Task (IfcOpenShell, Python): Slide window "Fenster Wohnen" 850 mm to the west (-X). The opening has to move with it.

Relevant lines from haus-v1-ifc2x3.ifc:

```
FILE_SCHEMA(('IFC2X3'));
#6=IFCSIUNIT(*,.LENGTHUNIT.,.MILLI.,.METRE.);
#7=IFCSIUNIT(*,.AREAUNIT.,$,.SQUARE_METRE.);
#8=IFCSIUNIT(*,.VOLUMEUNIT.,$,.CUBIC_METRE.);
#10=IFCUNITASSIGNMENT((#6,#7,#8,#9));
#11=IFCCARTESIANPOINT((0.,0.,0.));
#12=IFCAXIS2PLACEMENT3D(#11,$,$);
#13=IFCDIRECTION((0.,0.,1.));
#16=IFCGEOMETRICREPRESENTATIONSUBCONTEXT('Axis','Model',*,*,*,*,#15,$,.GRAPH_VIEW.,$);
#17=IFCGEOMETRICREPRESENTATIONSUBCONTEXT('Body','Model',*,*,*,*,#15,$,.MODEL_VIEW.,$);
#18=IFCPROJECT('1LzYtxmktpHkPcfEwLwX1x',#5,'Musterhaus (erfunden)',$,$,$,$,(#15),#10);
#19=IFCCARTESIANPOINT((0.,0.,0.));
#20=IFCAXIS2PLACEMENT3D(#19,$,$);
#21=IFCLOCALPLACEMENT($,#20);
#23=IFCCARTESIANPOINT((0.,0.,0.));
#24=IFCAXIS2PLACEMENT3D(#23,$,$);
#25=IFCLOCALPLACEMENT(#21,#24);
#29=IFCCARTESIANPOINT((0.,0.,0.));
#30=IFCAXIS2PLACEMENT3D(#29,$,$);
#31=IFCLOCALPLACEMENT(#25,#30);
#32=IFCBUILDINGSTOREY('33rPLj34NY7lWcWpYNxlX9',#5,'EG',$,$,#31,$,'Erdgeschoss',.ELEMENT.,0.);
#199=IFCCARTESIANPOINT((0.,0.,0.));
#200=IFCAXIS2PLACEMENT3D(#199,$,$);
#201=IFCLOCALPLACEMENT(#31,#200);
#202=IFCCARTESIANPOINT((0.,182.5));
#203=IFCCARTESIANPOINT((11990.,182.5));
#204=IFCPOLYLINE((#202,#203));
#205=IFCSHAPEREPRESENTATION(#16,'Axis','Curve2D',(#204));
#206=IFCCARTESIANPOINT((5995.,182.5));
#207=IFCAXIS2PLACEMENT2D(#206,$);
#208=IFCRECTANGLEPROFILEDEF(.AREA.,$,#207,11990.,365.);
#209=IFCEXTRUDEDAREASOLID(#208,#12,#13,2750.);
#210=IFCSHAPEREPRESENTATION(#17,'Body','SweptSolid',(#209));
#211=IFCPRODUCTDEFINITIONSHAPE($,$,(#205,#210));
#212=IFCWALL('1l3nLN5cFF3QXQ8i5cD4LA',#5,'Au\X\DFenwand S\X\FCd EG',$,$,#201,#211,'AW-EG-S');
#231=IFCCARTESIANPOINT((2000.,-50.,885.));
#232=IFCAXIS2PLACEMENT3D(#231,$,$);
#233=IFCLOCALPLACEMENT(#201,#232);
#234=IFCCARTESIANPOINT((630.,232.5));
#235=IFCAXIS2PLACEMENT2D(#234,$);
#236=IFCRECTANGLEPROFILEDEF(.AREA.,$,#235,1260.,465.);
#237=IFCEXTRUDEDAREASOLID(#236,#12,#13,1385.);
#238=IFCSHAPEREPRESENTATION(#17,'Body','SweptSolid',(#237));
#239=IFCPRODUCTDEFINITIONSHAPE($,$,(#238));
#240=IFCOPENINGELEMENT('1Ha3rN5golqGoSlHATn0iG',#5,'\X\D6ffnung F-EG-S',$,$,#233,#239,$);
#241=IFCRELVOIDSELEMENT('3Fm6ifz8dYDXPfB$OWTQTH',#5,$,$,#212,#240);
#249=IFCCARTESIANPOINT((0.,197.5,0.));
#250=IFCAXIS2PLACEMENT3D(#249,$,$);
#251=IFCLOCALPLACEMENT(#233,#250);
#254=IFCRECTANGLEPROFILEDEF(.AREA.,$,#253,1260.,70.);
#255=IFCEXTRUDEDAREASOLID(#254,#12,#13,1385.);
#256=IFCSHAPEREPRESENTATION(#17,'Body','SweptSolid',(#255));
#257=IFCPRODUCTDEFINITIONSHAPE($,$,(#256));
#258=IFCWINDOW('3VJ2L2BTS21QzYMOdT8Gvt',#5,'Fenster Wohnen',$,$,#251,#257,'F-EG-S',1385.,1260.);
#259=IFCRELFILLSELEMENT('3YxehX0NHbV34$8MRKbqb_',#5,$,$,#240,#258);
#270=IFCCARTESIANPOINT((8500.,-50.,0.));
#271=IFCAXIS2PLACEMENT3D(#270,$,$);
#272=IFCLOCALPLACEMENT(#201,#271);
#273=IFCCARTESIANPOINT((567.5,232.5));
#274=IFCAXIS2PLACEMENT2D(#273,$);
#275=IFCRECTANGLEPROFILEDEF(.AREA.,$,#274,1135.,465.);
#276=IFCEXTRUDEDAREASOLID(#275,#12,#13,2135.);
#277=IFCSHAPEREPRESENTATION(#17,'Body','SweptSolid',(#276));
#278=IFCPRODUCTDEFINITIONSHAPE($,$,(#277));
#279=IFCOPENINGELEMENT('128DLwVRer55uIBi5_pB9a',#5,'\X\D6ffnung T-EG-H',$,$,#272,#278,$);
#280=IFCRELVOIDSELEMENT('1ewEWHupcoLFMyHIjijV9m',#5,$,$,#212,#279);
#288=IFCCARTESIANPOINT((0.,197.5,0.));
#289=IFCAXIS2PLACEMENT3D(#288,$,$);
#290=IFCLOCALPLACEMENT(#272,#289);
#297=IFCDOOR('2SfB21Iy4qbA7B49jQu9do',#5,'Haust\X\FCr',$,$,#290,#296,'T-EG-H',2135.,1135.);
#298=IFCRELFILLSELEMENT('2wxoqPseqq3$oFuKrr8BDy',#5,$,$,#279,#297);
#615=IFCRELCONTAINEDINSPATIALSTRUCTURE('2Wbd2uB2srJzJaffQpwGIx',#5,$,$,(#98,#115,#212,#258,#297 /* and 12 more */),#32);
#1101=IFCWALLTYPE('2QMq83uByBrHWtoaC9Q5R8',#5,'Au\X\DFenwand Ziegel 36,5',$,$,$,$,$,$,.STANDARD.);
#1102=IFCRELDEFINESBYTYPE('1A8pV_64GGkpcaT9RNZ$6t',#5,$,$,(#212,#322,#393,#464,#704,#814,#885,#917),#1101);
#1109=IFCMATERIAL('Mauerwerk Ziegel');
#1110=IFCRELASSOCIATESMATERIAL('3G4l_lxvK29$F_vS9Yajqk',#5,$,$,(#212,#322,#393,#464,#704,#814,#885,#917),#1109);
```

```python
import ifcopenshell
import ifcopenshell.api.geometry
import ifcopenshell.util.placement
import ifcopenshell.util.unit

model = ifcopenshell.open("haus-v1-ifc2x3.ifc")
unit_scale = ifcopenshell.util.unit.calculate_unit_scale(model)

window = model.by_id(258)
opening = window.FillsVoids[0].RelatingOpeningElement
wall = opening.VoidsElements[0].RelatingBuildingElement

wall_matrix = ifcopenshell.util.placement.get_local_placement(wall.ObjectPlacement)
shift = wall_matrix[:3, 0] * -0.85 / unit_scale
before = ifcopenshell.util.placement.get_local_placement(window.ObjectPlacement)[:3, 3].copy()

# The window is placed relative to its opening, so it follows when the opening moves.
matrix = ifcopenshell.util.placement.get_local_placement(opening.ObjectPlacement)
matrix[:3, 3] += shift
ifcopenshell.api.geometry.edit_object_placement(
    model, product=opening, matrix=matrix, is_si=False, should_transform_children=True
)

after = ifcopenshell.util.placement.get_local_placement(window.ObjectPlacement)[:3, 3]
print("window moved by", (after - before).round(3) + 0.0)

model.write("haus-v1-ifc2x3-out.ifc")
```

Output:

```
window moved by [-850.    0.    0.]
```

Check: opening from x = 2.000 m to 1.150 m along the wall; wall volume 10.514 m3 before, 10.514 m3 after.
